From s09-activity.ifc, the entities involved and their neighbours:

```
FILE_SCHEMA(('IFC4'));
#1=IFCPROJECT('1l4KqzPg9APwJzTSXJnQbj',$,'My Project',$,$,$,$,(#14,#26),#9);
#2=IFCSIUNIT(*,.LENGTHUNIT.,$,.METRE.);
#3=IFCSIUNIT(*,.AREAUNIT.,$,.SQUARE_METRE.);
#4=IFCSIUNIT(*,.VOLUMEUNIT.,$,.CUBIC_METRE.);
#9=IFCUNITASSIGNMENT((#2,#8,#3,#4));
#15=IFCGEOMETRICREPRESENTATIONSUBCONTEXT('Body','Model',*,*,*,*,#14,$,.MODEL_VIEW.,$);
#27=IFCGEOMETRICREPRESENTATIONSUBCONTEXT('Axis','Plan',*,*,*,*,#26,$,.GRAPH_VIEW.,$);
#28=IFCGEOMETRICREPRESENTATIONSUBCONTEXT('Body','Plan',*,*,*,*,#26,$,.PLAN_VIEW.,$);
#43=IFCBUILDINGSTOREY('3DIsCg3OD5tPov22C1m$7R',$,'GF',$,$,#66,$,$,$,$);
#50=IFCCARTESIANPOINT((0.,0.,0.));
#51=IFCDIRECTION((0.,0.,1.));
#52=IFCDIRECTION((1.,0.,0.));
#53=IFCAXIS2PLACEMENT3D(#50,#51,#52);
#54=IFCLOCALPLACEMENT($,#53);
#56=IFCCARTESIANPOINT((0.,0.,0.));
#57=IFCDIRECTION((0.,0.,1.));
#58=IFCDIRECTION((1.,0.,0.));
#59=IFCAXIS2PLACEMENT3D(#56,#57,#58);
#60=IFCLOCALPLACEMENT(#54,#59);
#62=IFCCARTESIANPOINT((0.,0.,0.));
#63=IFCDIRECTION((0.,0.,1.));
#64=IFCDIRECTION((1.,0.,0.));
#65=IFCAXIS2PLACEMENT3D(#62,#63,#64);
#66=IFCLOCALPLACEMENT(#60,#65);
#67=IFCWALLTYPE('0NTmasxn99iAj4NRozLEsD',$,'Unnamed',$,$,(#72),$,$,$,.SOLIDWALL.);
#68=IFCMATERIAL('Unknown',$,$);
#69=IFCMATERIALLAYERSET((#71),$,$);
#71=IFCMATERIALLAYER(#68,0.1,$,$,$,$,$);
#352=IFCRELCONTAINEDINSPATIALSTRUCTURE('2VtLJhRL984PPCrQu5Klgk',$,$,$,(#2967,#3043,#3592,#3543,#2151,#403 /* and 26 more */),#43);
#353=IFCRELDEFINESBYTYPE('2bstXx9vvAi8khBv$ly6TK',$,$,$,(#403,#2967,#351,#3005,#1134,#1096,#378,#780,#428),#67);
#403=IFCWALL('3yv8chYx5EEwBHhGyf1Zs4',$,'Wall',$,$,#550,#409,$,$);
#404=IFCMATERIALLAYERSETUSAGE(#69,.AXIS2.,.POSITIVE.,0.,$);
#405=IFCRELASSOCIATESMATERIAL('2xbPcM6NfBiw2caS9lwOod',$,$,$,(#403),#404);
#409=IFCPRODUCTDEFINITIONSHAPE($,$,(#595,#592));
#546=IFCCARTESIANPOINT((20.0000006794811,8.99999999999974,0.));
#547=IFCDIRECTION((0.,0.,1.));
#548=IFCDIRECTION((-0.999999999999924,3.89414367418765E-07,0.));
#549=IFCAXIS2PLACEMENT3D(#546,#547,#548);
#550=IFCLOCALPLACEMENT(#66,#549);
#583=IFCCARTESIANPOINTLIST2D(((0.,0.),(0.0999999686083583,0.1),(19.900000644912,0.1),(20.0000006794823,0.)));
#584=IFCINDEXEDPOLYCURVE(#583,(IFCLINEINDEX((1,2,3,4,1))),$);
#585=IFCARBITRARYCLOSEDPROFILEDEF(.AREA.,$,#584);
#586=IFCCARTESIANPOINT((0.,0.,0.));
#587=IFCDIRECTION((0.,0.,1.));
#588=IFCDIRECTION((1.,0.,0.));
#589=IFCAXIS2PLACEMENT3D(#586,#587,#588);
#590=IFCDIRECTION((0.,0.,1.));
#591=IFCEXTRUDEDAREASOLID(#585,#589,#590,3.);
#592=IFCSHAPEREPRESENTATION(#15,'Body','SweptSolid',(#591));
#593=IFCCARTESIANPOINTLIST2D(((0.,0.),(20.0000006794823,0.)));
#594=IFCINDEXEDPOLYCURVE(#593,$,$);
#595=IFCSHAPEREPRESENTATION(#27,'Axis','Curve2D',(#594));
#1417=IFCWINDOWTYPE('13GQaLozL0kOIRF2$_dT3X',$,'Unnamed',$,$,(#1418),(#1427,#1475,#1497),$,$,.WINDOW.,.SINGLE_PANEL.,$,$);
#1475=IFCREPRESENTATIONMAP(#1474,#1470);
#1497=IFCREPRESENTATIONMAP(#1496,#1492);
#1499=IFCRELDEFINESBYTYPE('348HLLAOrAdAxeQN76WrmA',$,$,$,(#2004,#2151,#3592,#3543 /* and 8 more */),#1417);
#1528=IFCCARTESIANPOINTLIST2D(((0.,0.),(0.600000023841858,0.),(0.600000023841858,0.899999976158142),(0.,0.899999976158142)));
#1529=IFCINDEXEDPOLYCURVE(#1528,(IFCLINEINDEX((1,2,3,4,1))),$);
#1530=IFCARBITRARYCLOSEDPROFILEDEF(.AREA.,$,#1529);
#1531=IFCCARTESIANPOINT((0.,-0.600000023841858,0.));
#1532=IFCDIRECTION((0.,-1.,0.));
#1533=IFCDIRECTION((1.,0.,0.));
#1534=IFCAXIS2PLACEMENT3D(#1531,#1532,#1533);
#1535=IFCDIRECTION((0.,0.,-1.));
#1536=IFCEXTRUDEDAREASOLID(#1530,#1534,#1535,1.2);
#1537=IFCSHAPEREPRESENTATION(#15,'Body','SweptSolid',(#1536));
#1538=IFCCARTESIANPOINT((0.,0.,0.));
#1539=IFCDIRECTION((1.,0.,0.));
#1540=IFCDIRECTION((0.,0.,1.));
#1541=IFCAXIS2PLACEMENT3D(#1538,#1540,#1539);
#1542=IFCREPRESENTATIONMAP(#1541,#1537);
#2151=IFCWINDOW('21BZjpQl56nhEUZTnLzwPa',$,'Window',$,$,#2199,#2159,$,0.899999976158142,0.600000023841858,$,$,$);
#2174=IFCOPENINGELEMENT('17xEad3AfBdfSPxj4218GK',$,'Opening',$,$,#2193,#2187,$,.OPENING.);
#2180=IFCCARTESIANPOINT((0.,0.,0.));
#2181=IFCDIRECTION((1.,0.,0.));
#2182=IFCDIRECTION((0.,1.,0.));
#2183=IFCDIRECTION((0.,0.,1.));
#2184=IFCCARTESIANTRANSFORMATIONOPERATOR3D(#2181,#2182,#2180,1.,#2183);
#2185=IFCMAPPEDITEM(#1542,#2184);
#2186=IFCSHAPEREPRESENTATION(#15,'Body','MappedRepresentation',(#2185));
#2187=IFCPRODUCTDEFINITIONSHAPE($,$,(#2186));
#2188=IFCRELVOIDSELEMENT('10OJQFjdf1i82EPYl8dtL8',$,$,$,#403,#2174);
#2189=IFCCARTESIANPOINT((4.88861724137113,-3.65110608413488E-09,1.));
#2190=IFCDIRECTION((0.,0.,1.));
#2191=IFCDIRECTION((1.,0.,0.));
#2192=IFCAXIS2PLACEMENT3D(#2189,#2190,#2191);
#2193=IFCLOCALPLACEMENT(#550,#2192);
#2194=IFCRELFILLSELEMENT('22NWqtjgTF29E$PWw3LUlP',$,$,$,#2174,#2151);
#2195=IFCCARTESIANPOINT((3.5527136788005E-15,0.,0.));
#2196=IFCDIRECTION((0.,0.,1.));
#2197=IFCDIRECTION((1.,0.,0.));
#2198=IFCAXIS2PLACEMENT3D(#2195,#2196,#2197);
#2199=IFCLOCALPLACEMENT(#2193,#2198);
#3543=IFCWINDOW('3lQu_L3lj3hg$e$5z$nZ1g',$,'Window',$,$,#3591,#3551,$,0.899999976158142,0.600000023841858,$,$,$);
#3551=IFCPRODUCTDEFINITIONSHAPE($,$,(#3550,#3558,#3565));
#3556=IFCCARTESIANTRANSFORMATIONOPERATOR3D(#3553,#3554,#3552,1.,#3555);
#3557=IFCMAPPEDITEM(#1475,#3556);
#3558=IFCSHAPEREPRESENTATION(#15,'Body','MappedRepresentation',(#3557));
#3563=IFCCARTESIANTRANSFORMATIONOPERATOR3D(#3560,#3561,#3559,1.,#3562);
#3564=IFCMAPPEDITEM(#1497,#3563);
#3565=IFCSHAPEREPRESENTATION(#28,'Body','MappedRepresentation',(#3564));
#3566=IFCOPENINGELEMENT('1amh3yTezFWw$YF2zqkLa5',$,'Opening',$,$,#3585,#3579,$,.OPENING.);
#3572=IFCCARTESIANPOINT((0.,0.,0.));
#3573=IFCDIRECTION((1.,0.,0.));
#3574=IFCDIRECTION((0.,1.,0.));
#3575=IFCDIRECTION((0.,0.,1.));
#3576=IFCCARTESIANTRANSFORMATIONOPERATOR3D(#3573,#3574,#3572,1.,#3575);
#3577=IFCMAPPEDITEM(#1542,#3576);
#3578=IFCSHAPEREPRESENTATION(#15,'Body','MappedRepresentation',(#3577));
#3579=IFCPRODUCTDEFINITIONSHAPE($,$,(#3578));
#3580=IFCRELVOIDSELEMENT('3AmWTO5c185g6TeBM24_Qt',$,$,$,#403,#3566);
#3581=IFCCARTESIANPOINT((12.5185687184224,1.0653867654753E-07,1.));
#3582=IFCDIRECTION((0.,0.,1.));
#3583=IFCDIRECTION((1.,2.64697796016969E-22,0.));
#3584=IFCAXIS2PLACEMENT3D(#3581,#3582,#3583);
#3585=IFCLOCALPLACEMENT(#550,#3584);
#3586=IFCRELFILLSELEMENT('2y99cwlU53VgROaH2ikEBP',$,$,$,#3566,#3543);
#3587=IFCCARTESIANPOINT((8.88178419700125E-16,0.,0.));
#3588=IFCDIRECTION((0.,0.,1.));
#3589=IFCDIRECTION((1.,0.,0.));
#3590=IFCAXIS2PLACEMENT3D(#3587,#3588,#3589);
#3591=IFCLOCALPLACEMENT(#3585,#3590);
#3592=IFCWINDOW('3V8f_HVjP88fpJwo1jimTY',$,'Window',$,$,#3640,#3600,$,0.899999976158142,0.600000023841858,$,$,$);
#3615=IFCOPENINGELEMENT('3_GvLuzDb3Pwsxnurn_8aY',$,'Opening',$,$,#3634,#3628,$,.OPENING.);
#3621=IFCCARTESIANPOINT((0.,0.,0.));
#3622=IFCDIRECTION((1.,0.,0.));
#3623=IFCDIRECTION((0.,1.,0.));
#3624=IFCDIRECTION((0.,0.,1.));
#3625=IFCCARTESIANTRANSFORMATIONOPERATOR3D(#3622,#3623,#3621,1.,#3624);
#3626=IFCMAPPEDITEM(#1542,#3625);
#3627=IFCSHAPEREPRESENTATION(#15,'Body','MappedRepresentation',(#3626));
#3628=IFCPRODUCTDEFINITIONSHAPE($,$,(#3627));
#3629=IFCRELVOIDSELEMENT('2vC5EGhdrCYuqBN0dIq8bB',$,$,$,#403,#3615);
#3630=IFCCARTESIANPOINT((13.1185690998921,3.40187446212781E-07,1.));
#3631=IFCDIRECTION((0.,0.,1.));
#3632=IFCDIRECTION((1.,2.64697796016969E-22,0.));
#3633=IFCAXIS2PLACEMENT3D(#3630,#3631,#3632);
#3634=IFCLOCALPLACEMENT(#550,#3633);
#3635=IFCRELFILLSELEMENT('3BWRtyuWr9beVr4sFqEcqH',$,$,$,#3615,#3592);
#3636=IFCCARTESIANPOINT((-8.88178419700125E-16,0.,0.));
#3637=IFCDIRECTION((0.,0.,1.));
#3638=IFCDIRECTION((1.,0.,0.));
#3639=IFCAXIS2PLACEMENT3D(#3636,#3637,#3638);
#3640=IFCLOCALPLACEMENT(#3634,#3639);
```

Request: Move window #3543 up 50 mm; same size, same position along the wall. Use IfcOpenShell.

```python
import numpy as np
import ifcopenshell
import ifcopenshell.api.geometry
import ifcopenshell.util.placement
import ifcopenshell.util.unit

model = ifcopenshell.open("s09-activity.ifc")
unit_scale = ifcopenshell.util.unit.calculate_unit_scale(model)

window = model.by_id(3543)
opening = window.FillsVoids[0].RelatingOpeningElement
dz = 0.05

shift = np.array([0.0, 0.0, dz])
# The window is placed relative to its opening, so it follows when the opening moves.
matrix = ifcopenshell.util.placement.get_local_placement(opening.ObjectPlacement)
matrix[:3, 3] += shift
ifcopenshell.api.geometry.edit_object_placement(
    model, product=opening, matrix=matrix, is_si=False, should_transform_children=True
)

print(f"moved by {dz * unit_scale:+.3f} m")

model.write("s09-activity_updated.ifc")
```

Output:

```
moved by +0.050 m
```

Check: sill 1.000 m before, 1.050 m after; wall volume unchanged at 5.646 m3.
